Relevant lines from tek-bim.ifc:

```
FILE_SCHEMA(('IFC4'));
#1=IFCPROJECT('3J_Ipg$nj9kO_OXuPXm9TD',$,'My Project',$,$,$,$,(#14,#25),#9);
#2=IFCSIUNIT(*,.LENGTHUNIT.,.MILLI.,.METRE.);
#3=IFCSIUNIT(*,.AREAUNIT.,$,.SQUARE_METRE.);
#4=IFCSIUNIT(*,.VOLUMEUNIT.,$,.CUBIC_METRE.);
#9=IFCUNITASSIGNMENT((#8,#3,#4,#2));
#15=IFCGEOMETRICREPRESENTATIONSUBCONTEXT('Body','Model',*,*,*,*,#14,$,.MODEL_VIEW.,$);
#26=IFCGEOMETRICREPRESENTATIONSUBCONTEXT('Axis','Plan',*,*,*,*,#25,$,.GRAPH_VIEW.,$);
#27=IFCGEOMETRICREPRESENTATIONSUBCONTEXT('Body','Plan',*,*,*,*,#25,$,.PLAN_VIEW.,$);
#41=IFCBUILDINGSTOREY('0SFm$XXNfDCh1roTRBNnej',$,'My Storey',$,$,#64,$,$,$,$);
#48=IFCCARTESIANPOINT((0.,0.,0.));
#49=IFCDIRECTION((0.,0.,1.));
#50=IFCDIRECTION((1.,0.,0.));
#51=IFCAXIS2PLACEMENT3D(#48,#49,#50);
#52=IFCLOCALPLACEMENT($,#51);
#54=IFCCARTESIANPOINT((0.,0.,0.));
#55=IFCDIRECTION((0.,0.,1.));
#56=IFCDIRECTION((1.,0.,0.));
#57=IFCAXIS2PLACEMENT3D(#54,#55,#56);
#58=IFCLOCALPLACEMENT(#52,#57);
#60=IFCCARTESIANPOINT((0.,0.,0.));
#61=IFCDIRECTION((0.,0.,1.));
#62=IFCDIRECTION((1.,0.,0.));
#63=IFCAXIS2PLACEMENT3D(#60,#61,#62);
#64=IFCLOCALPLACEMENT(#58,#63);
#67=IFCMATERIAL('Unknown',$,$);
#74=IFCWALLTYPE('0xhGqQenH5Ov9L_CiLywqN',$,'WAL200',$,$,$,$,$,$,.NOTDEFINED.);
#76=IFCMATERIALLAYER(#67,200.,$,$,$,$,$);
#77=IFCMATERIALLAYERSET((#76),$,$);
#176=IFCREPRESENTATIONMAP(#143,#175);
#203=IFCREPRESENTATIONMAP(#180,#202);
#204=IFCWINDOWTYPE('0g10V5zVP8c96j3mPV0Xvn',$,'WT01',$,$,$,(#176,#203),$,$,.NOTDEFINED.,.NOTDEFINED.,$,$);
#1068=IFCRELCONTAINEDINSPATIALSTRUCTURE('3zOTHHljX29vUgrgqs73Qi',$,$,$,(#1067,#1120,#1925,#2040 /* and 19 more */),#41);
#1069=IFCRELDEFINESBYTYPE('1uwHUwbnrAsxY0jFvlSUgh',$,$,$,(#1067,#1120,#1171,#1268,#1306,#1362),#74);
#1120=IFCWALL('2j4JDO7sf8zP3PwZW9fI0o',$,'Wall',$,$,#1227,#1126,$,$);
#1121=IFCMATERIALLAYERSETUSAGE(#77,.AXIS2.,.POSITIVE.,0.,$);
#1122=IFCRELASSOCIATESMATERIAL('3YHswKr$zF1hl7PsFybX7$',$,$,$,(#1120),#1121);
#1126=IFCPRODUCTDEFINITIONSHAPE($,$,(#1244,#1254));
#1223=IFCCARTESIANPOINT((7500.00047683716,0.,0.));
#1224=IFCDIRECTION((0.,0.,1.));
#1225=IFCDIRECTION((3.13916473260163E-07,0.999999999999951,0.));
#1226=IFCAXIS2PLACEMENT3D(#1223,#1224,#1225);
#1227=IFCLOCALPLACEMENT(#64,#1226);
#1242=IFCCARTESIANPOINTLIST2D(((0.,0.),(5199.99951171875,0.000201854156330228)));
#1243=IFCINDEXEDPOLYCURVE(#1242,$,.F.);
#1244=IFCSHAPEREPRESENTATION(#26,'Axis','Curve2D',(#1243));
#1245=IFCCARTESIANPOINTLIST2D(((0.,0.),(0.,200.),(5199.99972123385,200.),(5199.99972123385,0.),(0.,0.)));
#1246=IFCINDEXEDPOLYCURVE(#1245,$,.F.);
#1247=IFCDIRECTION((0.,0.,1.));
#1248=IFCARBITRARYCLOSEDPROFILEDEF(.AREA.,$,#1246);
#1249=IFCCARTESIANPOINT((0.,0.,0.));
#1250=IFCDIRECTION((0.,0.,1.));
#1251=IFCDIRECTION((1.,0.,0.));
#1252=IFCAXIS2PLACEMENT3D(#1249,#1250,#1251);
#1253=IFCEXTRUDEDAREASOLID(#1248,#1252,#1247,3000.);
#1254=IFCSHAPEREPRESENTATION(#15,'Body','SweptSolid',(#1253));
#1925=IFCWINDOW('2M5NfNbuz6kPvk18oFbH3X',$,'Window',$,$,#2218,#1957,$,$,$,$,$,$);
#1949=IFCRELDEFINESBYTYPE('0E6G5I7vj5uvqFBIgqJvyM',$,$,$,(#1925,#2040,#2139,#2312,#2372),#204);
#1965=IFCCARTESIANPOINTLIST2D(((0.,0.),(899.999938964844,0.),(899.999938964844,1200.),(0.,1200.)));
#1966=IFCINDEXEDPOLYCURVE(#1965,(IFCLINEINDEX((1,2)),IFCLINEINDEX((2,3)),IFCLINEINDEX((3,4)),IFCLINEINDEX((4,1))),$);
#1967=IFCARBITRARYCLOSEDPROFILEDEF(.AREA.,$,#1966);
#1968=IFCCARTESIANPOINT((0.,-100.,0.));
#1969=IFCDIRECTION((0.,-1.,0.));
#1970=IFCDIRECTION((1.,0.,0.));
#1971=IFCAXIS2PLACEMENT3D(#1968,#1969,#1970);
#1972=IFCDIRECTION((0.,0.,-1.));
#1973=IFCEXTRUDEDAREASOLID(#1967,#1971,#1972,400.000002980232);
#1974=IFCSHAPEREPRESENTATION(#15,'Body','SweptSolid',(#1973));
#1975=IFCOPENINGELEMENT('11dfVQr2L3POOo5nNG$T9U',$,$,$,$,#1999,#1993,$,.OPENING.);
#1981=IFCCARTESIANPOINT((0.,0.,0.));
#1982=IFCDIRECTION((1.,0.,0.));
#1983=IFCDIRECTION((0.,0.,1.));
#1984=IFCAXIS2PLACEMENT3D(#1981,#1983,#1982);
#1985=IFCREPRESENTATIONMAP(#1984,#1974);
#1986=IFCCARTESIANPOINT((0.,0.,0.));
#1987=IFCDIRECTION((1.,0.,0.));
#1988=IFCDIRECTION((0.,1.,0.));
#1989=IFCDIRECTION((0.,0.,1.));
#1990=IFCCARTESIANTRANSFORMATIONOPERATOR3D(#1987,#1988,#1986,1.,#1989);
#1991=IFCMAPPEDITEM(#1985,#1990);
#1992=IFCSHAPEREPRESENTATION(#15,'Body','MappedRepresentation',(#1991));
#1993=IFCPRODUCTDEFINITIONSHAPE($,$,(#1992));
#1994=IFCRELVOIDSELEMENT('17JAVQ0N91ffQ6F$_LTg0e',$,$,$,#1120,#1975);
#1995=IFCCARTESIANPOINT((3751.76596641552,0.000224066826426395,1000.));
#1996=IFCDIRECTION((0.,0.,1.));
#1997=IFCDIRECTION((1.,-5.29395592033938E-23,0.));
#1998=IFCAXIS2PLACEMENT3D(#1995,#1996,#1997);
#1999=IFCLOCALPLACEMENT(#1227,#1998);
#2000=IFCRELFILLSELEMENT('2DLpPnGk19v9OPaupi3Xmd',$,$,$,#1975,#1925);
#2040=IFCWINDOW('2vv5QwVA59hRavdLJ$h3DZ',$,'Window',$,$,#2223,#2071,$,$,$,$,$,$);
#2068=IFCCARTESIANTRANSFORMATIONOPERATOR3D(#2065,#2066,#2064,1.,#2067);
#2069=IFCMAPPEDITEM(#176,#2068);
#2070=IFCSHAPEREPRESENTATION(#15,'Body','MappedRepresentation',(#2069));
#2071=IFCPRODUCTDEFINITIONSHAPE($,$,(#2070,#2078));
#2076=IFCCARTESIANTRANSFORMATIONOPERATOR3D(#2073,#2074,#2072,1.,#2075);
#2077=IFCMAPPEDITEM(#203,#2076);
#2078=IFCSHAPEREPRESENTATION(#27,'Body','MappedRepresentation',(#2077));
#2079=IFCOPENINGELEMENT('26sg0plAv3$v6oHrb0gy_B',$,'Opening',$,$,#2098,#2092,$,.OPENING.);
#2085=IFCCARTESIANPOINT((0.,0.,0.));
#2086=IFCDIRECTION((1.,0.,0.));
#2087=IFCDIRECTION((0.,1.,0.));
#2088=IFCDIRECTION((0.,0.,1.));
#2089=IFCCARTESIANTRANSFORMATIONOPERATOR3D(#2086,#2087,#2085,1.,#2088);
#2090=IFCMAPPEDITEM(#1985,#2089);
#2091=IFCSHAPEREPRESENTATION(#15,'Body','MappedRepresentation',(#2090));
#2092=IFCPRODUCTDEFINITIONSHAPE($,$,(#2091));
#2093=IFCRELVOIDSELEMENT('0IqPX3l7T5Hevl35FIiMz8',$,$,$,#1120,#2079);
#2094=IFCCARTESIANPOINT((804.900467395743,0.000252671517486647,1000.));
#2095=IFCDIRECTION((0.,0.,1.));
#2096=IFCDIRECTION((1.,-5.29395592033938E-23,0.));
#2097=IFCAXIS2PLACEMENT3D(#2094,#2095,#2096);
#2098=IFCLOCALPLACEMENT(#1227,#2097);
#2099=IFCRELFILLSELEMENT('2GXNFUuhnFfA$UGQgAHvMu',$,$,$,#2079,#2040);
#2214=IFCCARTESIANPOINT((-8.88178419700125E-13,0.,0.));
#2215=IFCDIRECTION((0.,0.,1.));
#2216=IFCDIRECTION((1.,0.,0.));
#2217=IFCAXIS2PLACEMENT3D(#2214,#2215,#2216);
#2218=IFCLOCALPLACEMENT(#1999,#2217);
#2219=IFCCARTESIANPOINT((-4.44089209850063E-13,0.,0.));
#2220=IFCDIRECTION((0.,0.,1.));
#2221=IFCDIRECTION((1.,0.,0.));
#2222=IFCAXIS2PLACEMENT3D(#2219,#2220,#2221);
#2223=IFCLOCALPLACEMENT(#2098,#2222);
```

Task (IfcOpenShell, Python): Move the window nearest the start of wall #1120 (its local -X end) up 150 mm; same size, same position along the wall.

```python
import numpy as np
import ifcopenshell
import ifcopenshell.api.geometry
import ifcopenshell.util.placement
import ifcopenshell.util.unit

model = ifcopenshell.open("tek-bim.ifc")
unit_scale = ifcopenshell.util.unit.calculate_unit_scale(model)

window = model.by_guid("2vv5QwVA59hRavdLJ$h3DZ")
opening = window.FillsVoids[0].RelatingOpeningElement
dz = 0.15 / unit_scale

shift = np.array([0.0, 0.0, dz])
# The window is placed relative to its opening, so it follows when the opening moves.
matrix = ifcopenshell.util.placement.get_local_placement(opening.ObjectPlacement)
matrix[:3, 3] += shift
ifcopenshell.api.geometry.edit_object_placement(
    model, product=opening, matrix=matrix, is_si=False, should_transform_children=True
)

print(f"moved by {dz * unit_scale:+.3f} m")

model.write("tek-bim_v2.ifc")
```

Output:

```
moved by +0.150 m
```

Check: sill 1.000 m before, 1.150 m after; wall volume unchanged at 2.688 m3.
